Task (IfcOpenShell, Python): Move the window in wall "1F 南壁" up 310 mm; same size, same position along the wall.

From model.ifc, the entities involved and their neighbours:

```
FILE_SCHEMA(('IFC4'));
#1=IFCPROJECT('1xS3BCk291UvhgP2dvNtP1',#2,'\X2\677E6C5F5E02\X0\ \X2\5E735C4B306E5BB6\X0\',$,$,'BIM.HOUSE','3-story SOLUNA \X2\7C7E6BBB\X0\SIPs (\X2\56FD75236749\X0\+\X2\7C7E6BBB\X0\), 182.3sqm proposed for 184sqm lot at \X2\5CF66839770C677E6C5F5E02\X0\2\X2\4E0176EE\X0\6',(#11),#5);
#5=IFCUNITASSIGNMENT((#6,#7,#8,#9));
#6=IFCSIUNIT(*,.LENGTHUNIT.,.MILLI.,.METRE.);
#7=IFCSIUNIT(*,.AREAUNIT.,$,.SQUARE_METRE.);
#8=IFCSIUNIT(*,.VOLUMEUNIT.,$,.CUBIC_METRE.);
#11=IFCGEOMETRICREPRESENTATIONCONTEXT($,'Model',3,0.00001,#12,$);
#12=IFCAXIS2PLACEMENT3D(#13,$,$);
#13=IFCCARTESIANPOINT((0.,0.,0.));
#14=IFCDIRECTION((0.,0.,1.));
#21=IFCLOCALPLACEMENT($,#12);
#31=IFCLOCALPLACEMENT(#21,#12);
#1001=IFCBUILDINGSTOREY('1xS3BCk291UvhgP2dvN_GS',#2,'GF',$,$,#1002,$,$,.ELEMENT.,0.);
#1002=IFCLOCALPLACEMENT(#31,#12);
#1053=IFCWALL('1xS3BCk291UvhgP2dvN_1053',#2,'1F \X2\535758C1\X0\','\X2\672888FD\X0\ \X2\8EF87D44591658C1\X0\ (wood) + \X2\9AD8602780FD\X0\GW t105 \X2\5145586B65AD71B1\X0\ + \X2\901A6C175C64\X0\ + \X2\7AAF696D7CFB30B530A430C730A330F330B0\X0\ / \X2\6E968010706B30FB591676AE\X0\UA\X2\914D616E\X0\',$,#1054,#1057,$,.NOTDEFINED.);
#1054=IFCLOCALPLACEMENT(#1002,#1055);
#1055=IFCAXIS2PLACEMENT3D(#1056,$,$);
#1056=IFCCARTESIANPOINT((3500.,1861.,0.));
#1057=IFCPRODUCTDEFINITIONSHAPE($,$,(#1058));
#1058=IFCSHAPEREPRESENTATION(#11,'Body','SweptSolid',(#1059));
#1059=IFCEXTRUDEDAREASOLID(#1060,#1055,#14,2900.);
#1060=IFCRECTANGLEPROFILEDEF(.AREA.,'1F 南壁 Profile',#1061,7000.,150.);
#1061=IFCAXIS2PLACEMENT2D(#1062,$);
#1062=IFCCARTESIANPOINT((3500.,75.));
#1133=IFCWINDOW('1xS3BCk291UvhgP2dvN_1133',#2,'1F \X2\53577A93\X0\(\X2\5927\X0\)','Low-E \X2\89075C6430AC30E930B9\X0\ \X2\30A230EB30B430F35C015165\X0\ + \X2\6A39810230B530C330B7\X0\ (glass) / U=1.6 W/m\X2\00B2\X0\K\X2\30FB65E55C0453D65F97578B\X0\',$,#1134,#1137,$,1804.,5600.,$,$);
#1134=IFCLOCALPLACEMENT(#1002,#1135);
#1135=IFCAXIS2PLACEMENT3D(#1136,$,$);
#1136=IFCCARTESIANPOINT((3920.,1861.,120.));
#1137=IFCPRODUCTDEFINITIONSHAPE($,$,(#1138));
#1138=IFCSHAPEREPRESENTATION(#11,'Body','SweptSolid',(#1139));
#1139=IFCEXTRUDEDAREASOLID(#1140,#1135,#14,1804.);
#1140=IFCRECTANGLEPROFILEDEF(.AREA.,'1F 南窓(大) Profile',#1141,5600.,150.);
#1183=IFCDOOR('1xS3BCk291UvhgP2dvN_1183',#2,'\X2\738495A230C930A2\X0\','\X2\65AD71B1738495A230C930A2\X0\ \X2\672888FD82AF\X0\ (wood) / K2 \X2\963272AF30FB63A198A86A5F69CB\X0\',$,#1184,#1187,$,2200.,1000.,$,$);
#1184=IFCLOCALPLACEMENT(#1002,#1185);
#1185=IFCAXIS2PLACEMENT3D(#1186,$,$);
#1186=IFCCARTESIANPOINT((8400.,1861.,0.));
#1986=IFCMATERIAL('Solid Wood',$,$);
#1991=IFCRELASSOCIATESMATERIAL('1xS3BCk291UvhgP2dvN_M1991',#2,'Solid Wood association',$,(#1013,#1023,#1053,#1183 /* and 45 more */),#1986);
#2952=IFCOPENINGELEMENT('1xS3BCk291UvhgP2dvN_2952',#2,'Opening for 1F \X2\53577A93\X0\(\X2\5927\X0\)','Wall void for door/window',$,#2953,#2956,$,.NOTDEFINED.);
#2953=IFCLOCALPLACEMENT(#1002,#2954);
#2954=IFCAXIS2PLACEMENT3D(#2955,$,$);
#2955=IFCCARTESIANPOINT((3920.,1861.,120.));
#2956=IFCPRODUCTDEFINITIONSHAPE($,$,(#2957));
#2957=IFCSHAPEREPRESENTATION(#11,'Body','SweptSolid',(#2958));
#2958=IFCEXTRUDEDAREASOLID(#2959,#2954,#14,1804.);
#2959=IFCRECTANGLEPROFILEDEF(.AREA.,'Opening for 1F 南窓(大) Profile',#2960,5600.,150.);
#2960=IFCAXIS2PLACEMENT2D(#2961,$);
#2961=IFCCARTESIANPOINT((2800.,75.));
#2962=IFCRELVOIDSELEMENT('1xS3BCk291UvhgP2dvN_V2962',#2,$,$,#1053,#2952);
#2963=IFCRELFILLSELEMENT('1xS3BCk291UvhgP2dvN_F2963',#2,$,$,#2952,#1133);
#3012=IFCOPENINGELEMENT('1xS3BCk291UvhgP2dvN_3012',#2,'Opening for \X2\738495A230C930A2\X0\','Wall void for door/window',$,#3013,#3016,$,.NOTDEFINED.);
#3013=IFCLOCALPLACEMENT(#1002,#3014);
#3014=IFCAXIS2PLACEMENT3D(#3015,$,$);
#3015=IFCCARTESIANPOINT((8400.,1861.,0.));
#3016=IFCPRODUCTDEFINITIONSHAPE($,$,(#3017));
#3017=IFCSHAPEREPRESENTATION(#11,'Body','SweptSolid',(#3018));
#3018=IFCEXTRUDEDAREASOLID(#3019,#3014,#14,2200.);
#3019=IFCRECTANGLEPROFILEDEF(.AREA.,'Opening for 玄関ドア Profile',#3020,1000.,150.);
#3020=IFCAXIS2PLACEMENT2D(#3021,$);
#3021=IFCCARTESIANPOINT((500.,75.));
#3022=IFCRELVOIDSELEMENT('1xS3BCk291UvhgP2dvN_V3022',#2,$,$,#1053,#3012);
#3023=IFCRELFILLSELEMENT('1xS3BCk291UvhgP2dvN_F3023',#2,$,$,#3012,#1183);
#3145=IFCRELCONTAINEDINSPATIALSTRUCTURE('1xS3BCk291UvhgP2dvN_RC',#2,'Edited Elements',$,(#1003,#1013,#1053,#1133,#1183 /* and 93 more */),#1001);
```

```python
import numpy as np
import ifcopenshell
import ifcopenshell.api.geometry
import ifcopenshell.util.placement
import ifcopenshell.util.unit

model = ifcopenshell.open("model.ifc")
unit_scale = ifcopenshell.util.unit.calculate_unit_scale(model)

window = model.by_guid("1xS3BCk291UvhgP2dvN_1133")
opening = window.FillsVoids[0].RelatingOpeningElement
dz = 0.31 / unit_scale

shift = np.array([0.0, 0.0, dz])
# The window is not placed relative to its opening, so move both.
for product in (opening, window):
    matrix = ifcopenshell.util.placement.get_local_placement(product.ObjectPlacement)
    matrix[:3, 3] += shift
    ifcopenshell.api.geometry.edit_object_placement(model, product=product, matrix=matrix, is_si=False)

print(f"moved by {dz * unit_scale:+.3f} m")

model.write("model_rev.ifc")
```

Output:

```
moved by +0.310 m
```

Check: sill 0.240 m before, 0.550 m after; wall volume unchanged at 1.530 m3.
